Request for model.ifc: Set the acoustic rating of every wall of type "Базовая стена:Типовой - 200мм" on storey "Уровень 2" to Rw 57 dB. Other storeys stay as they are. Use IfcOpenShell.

First a look at what the model holds.

```python
import ifcopenshell
import ifcopenshell.util.element

model = ifcopenshell.open("model.ifc")
print(model.schema)
storey = next(s for s in model.by_type("IfcBuildingStorey") if s.Name == "Уровень 2")
walls = [e for e in ifcopenshell.util.element.get_decomposition(storey) if e.is_a("IfcWall")]
seen = {}
for e in walls:
    element_type = ifcopenshell.util.element.get_type(e)
    key = (element_type.Name if element_type != e and element_type else None, ifcopenshell.util.element.get_pset(e, "Pset_WallCommon", "AcousticRating"))
    seen[key] = seen.get(key, 0) + 1
for (name, value), count in sorted(seen.items(), key=str):
    print(count, "x", name, "|", value)
```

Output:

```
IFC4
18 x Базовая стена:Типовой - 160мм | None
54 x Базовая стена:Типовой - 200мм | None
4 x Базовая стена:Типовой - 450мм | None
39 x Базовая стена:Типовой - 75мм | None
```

```python
import ifcopenshell
import ifcopenshell.api.pset
import ifcopenshell.util.element

model = ifcopenshell.open("model.ifc")

storey = next(s for s in model.by_type("IfcBuildingStorey") if s.Name == "Уровень 2")
walls = [e for e in ifcopenshell.util.element.get_decomposition(storey) if e.is_a("IfcWall")]

count = 0
for e in walls:
    element_type = ifcopenshell.util.element.get_type(e)
    if element_type in (None, e) or element_type.Name != "Базовая стена:Типовой - 200мм":
        continue
    # add_pset returns the element's existing set when there is one.
    pset = ifcopenshell.api.pset.add_pset(model, product=e, name="Pset_WallCommon")
    ifcopenshell.api.pset.edit_pset(model, pset=pset, properties={"AcousticRating": "Rw 57 dB"})
    count += 1

print(count, "walls updated")

model.write("model-out.ifc")
```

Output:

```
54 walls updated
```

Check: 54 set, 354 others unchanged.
